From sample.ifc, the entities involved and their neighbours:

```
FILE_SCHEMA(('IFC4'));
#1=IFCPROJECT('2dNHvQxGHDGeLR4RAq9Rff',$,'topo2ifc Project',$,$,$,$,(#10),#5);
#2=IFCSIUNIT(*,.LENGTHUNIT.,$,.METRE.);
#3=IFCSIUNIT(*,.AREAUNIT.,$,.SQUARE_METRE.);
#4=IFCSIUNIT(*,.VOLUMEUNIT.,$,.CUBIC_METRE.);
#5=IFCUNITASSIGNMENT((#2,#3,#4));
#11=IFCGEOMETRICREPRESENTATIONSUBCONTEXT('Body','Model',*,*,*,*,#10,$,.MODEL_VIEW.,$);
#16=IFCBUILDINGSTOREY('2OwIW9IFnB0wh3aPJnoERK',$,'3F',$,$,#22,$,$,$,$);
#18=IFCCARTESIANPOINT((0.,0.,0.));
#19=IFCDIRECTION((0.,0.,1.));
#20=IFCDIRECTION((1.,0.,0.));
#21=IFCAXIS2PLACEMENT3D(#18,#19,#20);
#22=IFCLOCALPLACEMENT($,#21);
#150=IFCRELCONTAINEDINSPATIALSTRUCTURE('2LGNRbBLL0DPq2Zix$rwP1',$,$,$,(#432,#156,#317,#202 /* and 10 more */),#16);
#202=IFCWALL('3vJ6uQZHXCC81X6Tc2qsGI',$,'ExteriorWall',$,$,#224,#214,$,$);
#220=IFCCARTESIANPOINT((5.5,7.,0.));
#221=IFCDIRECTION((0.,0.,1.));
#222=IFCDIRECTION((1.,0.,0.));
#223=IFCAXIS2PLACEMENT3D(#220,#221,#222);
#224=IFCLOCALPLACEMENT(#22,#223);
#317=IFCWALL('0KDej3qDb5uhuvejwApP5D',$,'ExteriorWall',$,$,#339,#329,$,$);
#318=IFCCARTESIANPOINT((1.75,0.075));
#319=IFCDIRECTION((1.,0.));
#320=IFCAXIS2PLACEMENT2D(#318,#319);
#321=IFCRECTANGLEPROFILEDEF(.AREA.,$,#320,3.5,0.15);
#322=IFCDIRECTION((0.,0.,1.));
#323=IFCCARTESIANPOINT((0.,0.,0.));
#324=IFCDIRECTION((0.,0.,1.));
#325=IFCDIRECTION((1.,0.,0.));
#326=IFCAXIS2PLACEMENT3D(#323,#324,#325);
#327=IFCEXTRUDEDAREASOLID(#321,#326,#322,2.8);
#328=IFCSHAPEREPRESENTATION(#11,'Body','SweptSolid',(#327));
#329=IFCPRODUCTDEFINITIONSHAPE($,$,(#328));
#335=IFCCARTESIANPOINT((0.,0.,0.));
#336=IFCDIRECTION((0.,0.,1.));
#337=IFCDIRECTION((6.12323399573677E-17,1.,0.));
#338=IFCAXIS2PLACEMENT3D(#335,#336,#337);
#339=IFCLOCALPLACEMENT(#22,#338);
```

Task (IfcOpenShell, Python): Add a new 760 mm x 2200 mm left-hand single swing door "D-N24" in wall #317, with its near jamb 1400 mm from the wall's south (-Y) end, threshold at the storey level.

```python
import numpy as np
import ifcopenshell
import ifcopenshell.api.feature
import ifcopenshell.api.geometry
import ifcopenshell.api.root
import ifcopenshell.api.spatial
import ifcopenshell.geom
import ifcopenshell.util.element
import ifcopenshell.util.placement
import ifcopenshell.util.representation
import ifcopenshell.util.shape
import ifcopenshell.util.unit

model = ifcopenshell.open("sample.ifc")
unit_scale = ifcopenshell.util.unit.calculate_unit_scale(model)
settings = ifcopenshell.geom.settings()


def volume(element):
    """Net volume in cubic metres, openings subtracted."""
    shape = ifcopenshell.geom.create_shape(settings, element)
    return ifcopenshell.util.shape.get_volume(shape.geometry)


wall = model.by_id(317)
storey = ifcopenshell.util.element.get_container(wall, ifc_class="IfcBuildingStorey")
context = ifcopenshell.util.representation.get_context(model, "Model", "Body", "MODEL_VIEW")
before = volume(wall)

width, height, from_end, sill = 0.76, 2.2, 1.4, 0.0  # metres

# The wall runs along its own X axis, and the end named is its -X end.
wall_shape = ifcopenshell.geom.create_shape(settings, wall)
x, y, z = ifcopenshell.util.shape.get_vertices(wall_shape.geometry).T
start = x.min() + from_end
face, thickness = float(y.min()), float(y.max() - y.min())
wall_matrix = ifcopenshell.util.placement.get_local_placement(wall.ObjectPlacement)
level = ifcopenshell.util.placement.get_local_placement(storey.ObjectPlacement)[2, 3]


def in_wall(x, y):
    """Placement at x, y metres in the wall's axes, at sill height."""
    matrix = wall_matrix.copy()
    matrix[:, 3] = wall_matrix @ np.array([x / unit_scale, y / unit_scale, 0.0, 1.0])
    matrix[2, 3] = level + sill / unit_scale
    return matrix


# Opening: a box that overshoots both wall faces by 50 mm.
opening = ifcopenshell.api.root.create_entity(model, ifc_class="IfcOpeningElement", predefined_type="OPENING")
box = ifcopenshell.api.geometry.add_wall_representation(
    model, context=context, length=width, height=height, thickness=thickness + 0.1
)
ifcopenshell.api.geometry.assign_representation(model, product=opening, representation=box)
ifcopenshell.api.geometry.edit_object_placement(model, product=opening, matrix=in_wall(start, face - 0.05), is_si=False)
ifcopenshell.api.feature.add_feature(model, feature=opening, element=wall)

door = ifcopenshell.api.root.create_entity(model, ifc_class="IfcDoor", name="D-N24", predefined_type="DOOR")
door.OverallWidth, door.OverallHeight = width / unit_scale, height / unit_scale
door.OperationType = "SINGLE_SWING_LEFT"
body = ifcopenshell.api.geometry.add_door_representation(
    model,
    context=context,
    overall_width=door.OverallWidth,
    overall_height=door.OverallHeight,
    operation_type="SINGLE_SWING_LEFT",
    lining_properties={"LiningDepth": thickness / unit_scale, "ThresholdDepth": thickness / unit_scale},
)
ifcopenshell.api.geometry.assign_representation(model, product=door, representation=body)
ifcopenshell.api.spatial.assign_container(model, products=[door], relating_structure=storey)
ifcopenshell.api.feature.add_filling(model, opening=opening, element=door)

# The lining spans the wall, so the door starts at the wall face.
ifcopenshell.api.geometry.edit_object_placement(model, product=door, matrix=in_wall(start, face), is_si=False)

after = volume(wall)

print(f"wall volume {before:.3f} -> {after:.3f} m3")

model.write("sample_rev.ifc")
```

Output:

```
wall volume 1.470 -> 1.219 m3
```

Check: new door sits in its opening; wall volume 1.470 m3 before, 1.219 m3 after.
